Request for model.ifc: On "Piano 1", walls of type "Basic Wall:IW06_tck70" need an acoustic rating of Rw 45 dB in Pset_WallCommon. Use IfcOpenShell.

First a look at what the model holds.

```python
import ifcopenshell
import ifcopenshell.util.element

model = ifcopenshell.open("model.ifc")
print(model.schema)
storey = next(s for s in model.by_type("IfcBuildingStorey") if s.Name == "Piano 1")
walls = [e for e in ifcopenshell.util.element.get_decomposition(storey) if e.is_a("IfcWall")]
seen = {}
for e in walls:
    element_type = ifcopenshell.util.element.get_type(e)
    key = (element_type.Name if element_type != e and element_type else None, ifcopenshell.util.element.get_pset(e, "Pset_WallCommon", "AcousticRating"))
    seen[key] = seen.get(key, 0) + 1
for (name, value), count in sorted(seen.items(), key=str):
    print(count, "x", name, "|", value)
```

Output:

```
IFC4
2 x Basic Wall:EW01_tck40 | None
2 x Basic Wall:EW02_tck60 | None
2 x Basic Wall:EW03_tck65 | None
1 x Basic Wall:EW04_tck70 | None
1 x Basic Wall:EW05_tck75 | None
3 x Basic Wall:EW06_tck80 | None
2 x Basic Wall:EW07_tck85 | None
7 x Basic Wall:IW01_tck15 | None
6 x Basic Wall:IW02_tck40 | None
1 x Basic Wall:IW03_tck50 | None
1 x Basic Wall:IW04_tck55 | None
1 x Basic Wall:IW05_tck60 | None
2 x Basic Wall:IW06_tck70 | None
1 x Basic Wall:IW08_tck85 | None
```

```python
import ifcopenshell
import ifcopenshell.api.pset
import ifcopenshell.util.element

model = ifcopenshell.open("model.ifc")

storey = next(s for s in model.by_type("IfcBuildingStorey") if s.Name == "Piano 1")
walls = [e for e in ifcopenshell.util.element.get_decomposition(storey) if e.is_a("IfcWall")]

count = 0
for e in walls:
    element_type = ifcopenshell.util.element.get_type(e)
    if element_type in (None, e) or element_type.Name != "Basic Wall:IW06_tck70":
        continue
    # add_pset returns the element's existing set when there is one.
    pset = ifcopenshell.api.pset.add_pset(model, product=e, name="Pset_WallCommon")
    ifcopenshell.api.pset.edit_pset(model, pset=pset, properties={"AcousticRating": "Rw 45 dB"})
    count += 1

print(count, "walls updated")

model.write("model_updated.ifc")
```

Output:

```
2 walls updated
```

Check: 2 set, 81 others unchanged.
